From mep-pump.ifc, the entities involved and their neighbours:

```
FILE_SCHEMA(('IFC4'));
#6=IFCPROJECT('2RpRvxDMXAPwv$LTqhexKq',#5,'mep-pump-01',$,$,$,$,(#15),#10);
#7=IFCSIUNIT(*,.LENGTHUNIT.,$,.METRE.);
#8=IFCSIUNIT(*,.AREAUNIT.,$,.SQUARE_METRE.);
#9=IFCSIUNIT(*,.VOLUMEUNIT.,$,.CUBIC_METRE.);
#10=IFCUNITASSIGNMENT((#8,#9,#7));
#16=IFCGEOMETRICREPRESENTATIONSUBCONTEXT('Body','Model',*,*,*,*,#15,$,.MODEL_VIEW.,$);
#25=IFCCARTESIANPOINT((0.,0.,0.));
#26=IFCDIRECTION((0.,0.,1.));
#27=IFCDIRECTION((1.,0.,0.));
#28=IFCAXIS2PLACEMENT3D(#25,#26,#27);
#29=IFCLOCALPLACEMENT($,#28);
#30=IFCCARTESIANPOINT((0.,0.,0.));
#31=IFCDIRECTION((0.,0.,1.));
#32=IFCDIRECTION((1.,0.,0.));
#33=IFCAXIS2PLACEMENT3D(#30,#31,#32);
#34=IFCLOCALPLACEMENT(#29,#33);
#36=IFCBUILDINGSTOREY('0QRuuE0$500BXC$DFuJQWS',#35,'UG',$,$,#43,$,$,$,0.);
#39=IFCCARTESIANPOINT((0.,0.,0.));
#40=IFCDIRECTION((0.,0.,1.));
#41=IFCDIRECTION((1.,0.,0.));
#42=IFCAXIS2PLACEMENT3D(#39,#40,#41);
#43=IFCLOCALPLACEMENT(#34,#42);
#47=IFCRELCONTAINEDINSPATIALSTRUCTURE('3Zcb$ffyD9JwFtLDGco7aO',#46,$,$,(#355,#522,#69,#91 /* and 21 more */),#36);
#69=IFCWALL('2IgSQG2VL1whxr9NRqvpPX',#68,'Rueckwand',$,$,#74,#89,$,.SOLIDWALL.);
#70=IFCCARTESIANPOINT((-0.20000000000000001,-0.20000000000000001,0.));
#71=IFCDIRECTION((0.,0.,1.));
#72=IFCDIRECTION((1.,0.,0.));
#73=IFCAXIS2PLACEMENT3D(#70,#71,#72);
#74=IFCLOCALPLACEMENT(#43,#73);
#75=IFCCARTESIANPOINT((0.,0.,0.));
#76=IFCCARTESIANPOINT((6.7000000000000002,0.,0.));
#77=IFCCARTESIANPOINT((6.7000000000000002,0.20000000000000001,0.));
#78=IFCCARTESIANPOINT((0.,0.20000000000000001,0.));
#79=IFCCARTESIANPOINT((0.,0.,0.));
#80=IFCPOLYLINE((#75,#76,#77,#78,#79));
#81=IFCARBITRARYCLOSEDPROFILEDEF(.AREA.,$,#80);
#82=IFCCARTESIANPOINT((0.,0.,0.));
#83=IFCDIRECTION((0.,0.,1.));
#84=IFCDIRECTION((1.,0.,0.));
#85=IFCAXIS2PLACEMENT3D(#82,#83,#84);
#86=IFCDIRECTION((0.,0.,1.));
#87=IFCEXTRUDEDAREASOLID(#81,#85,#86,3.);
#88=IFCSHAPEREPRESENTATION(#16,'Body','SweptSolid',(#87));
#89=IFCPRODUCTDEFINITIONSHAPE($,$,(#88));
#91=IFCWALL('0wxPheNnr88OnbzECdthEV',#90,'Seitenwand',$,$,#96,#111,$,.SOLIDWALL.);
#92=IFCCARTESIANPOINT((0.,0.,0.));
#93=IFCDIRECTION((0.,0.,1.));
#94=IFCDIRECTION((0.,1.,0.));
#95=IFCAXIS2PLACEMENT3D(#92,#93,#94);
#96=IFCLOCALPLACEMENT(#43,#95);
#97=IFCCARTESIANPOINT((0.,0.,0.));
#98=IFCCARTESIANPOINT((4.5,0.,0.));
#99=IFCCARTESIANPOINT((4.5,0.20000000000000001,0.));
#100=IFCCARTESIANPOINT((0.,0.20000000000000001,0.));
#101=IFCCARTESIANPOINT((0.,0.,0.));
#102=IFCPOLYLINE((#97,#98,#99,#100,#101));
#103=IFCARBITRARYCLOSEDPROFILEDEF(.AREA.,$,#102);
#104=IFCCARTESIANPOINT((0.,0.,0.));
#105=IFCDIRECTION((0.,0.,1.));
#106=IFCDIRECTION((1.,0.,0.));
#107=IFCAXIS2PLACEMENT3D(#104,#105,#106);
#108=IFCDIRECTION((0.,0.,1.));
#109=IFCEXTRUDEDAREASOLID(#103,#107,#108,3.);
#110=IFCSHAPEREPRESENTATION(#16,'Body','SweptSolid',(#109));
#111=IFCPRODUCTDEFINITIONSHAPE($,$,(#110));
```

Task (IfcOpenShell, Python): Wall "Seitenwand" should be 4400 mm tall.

```python
import ifcopenshell
import ifcopenshell.geom
import ifcopenshell.util.representation
import ifcopenshell.util.shape
import ifcopenshell.util.unit

model = ifcopenshell.open("mep-pump.ifc")
unit_scale = ifcopenshell.util.unit.calculate_unit_scale(model)
settings = ifcopenshell.geom.settings()


def volume(element):
    """Net volume in cubic metres, openings subtracted."""
    shape = ifcopenshell.geom.create_shape(settings, element)
    return ifcopenshell.util.shape.get_volume(shape.geometry)


wall = model.by_guid("0wxPheNnr88OnbzECdthEV")
before = volume(wall)

body = ifcopenshell.util.representation.get_representation(wall, "Model", "Body")
solid = body.Items[0]
old_height = solid.Depth
solid.Depth = 4.4 / unit_scale
after = volume(wall)

print(f"height {old_height:g} -> {solid.Depth:g}, volume {before:.3f} -> {after:.3f} m3")

model.write("mep-pump_rev.ifc")
```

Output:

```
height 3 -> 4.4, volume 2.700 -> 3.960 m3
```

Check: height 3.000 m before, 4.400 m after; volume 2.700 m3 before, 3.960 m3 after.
